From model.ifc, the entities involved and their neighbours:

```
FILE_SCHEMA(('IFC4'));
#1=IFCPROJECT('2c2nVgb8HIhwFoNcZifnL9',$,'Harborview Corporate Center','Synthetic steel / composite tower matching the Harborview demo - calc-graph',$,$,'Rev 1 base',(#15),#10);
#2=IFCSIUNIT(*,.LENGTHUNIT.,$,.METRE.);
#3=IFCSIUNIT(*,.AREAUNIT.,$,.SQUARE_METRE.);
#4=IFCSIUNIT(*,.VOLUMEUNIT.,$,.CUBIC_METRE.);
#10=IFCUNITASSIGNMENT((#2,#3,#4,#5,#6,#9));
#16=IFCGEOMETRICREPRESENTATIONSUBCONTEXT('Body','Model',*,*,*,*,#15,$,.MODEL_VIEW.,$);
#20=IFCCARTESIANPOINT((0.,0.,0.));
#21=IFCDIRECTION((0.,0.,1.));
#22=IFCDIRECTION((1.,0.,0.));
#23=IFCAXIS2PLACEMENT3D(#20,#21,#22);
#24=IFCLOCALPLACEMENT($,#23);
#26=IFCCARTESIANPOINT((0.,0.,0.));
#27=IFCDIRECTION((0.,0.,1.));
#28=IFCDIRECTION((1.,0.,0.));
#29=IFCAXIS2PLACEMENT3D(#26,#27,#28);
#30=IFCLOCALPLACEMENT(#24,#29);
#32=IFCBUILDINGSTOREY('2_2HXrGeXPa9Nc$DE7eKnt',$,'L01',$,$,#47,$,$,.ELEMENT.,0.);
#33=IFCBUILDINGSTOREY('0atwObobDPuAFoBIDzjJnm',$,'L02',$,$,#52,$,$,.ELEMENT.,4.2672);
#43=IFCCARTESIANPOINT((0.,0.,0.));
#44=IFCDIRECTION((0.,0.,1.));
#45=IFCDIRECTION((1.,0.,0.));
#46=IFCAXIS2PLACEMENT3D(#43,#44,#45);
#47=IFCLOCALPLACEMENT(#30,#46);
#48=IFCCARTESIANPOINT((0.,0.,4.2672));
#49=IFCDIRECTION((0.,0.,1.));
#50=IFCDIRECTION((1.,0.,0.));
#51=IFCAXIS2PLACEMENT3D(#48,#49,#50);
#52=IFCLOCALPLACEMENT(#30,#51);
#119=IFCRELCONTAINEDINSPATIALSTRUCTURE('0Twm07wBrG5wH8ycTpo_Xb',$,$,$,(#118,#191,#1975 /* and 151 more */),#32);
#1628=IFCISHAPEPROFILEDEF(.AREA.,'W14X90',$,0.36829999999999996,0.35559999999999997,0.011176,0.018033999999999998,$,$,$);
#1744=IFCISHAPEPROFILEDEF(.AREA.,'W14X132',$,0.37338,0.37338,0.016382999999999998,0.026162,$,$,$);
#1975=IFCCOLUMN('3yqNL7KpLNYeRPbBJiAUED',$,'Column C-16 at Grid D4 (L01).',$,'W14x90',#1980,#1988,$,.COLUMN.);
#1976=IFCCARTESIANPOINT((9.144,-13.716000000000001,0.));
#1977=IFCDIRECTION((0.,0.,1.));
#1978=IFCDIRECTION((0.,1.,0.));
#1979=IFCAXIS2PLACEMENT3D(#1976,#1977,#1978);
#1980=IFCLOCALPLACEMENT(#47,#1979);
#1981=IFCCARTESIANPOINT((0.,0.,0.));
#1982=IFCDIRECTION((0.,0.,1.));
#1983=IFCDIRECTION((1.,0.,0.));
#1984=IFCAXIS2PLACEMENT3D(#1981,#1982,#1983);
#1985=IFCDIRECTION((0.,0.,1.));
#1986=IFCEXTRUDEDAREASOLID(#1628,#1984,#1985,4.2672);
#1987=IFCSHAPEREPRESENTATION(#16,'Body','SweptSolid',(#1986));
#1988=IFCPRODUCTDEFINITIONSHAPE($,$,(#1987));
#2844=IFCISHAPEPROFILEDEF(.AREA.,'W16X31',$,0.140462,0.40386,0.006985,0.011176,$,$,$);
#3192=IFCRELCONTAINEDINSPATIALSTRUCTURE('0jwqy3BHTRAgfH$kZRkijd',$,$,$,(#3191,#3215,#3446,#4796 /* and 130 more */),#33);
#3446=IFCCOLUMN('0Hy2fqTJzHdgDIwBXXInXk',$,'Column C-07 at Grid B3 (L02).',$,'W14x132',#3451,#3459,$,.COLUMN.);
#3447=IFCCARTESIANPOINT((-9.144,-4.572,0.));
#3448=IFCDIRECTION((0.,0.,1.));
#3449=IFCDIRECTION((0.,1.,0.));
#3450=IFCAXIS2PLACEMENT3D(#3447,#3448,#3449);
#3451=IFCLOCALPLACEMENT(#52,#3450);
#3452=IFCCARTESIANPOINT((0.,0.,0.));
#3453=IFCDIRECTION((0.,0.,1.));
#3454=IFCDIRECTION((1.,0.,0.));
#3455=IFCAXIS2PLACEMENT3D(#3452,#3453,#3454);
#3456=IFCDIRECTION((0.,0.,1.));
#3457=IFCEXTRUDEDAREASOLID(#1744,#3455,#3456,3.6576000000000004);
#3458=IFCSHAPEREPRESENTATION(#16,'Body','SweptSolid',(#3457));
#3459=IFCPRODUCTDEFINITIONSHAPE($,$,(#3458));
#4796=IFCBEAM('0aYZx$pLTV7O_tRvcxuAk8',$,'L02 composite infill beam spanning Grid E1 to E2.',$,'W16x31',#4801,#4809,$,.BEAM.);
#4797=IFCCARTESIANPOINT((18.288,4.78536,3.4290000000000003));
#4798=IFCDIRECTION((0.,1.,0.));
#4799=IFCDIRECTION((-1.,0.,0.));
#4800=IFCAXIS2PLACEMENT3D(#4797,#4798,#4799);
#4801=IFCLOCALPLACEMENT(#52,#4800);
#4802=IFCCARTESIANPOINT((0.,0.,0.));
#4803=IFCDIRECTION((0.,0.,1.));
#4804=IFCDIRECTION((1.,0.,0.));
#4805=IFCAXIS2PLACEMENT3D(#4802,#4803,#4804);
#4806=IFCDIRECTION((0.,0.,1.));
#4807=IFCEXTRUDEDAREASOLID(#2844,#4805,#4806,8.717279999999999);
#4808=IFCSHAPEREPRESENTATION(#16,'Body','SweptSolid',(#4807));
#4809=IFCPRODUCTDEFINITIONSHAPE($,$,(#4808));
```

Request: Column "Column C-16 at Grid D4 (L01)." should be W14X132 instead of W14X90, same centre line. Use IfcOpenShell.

```python
import ifcopenshell
import ifcopenshell.util.element
import ifcopenshell.util.representation

model = ifcopenshell.open("model.ifc")

member = model.by_id(1975)
source = next(p for p in model.by_type("IfcIShapeProfileDef") if p.ProfileName == "W14X132")

body = ifcopenshell.util.representation.get_representation(member, "Model", "Body")
solid = body.Items[0]
old_profile = solid.SweptArea

# Copy the section's sizes but keep this member's own profile position.
profile = ifcopenshell.util.element.copy(model, source)
profile.Position = old_profile.Position
solid.SweptArea = profile
if not model.get_total_inverses(old_profile):
    ifcopenshell.util.element.remove_deep2(model, old_profile)

print(solid.SweptArea)

model.write("model_v2.ifc")
```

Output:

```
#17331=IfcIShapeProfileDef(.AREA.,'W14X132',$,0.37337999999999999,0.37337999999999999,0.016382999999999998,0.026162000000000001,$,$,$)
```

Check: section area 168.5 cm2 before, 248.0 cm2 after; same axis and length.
